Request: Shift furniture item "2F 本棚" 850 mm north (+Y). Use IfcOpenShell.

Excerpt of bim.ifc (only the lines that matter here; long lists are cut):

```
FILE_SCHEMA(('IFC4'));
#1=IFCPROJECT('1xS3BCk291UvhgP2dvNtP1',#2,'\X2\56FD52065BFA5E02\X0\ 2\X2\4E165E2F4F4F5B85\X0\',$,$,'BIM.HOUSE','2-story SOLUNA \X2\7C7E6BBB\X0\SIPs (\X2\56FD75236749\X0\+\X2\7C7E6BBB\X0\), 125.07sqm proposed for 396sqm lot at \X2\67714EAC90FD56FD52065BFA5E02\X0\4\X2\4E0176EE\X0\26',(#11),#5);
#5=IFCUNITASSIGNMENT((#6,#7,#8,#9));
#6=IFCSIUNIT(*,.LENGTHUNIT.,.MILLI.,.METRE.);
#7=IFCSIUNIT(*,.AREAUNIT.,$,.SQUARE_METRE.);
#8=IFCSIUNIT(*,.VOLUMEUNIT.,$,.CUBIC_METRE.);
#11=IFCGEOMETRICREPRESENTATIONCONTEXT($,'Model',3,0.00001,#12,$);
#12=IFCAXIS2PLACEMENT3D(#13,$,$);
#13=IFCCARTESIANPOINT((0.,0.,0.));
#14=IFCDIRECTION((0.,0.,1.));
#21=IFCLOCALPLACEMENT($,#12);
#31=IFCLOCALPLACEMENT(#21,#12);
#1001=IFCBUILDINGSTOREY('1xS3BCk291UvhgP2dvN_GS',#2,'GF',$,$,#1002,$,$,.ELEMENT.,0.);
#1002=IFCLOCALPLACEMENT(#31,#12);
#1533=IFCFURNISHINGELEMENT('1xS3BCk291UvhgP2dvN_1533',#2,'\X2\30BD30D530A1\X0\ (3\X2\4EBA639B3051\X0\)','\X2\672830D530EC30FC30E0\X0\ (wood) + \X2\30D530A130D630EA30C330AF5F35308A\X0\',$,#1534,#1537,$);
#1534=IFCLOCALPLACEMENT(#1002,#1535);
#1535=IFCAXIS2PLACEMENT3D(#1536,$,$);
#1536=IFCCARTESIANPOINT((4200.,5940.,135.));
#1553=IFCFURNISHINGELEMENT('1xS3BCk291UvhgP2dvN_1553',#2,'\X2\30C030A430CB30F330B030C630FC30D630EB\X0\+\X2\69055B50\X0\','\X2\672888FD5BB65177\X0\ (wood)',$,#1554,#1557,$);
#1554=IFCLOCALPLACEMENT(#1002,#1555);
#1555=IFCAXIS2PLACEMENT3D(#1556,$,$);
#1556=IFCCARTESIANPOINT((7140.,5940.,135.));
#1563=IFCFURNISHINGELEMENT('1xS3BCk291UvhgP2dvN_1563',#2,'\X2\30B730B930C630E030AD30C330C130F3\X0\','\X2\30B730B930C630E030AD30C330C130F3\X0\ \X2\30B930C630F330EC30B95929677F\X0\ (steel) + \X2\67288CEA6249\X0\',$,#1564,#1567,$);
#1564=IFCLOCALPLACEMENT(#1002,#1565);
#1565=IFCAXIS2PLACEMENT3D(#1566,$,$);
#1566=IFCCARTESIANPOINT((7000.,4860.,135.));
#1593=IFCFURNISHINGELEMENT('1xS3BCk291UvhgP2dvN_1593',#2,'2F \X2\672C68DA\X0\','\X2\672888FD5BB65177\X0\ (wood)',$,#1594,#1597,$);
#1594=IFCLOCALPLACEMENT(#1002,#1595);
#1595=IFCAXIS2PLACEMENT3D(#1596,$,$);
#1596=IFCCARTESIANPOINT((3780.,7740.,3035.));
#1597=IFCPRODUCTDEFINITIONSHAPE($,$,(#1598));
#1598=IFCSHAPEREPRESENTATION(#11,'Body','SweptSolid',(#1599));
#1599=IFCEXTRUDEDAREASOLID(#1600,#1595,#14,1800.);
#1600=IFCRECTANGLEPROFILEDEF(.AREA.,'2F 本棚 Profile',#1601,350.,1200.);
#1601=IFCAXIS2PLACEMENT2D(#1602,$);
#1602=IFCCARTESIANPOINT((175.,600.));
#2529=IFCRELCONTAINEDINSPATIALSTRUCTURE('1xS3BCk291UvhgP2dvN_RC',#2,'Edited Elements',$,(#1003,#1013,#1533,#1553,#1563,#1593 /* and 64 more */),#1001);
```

```python
import ifcopenshell
import ifcopenshell.api.geometry
import ifcopenshell.util.placement
import ifcopenshell.util.unit

model = ifcopenshell.open("bim.ifc")
unit_scale = ifcopenshell.util.unit.calculate_unit_scale(model)

item = model.by_guid("1xS3BCk291UvhgP2dvN_1593")
matrix = ifcopenshell.util.placement.get_local_placement(item.ObjectPlacement)
matrix[1, 3] += 0.85 / unit_scale
ifcopenshell.api.geometry.edit_object_placement(model, product=item, matrix=matrix, is_si=False)

print(ifcopenshell.util.placement.get_local_placement(item.ObjectPlacement).round(3) + 0.0)

model.write("bim-out.ifc")
```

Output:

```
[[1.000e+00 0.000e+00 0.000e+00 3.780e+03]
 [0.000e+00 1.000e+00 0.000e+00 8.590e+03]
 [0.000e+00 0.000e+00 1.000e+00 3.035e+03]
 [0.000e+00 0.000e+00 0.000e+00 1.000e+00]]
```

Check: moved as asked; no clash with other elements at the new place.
